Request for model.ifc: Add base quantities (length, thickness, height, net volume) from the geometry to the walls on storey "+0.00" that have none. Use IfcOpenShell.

First a look at what the model holds.

```python
import ifcopenshell
import ifcopenshell.util.element
import ifcopenshell.util.unit

model = ifcopenshell.open("model.ifc")
print(model.schema)
for unit_type in ("LENGTHUNIT", "AREAUNIT", "VOLUMEUNIT"):
    print(unit_type, ifcopenshell.util.unit.calculate_unit_scale(model, unit_type))
storey = next(s for s in model.by_type("IfcBuildingStorey") if s.Name == "+0.00")
walls = [e for e in ifcopenshell.util.element.get_decomposition(storey) if e.is_a("IfcWall")]
for e in sorted(walls, key=lambda e: e.id()):
    print(e.id(), e.is_a(), e.Name, list(ifcopenshell.util.element.get_psets(e, qtos_only=True)), sep=" | ")
```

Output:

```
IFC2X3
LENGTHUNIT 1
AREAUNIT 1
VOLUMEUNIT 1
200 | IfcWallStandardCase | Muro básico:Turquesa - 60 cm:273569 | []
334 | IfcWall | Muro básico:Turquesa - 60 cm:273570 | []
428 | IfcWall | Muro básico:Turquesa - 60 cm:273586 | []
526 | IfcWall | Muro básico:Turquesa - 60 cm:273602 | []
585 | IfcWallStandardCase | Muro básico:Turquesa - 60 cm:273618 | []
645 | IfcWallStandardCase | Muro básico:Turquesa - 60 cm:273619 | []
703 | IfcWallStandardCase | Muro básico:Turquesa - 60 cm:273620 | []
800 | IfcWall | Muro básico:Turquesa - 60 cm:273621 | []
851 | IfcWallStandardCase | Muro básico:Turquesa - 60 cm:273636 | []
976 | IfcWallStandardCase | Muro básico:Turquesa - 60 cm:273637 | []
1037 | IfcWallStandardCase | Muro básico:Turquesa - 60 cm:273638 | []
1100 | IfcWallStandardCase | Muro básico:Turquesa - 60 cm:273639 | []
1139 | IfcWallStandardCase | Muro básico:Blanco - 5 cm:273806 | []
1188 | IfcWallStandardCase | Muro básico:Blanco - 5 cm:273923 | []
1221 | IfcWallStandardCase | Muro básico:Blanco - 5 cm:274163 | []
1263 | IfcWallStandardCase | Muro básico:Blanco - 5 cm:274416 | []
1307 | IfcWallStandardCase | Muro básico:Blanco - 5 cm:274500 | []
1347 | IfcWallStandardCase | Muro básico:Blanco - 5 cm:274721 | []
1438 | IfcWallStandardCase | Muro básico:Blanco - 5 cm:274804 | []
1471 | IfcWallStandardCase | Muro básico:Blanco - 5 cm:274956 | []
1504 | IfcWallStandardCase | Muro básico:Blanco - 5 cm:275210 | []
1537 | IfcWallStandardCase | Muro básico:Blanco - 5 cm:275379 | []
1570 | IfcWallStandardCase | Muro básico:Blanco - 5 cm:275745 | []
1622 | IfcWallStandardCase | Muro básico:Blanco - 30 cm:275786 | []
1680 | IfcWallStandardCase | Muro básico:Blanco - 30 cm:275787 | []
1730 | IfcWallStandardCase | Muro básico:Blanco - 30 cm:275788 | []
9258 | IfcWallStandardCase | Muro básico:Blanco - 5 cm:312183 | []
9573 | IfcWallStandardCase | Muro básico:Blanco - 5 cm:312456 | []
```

```python
import ifcopenshell
import ifcopenshell.api.pset
import ifcopenshell.geom
import ifcopenshell.util.element
import ifcopenshell.util.shape
import ifcopenshell.util.unit

model = ifcopenshell.open("model.ifc")
unit_scale = ifcopenshell.util.unit.calculate_unit_scale(model)
volume_scale = ifcopenshell.util.unit.calculate_unit_scale(model, "VOLUMEUNIT")
settings = ifcopenshell.geom.settings()

storey = next(s for s in model.by_type("IfcBuildingStorey") if s.Name == "+0.00")
walls = [e for e in ifcopenshell.util.element.get_decomposition(storey) if e.is_a("IfcWall")]

for e in sorted(walls, key=lambda e: e.id()):
    if ifcopenshell.util.element.get_psets(e, qtos_only=True, should_inherit=False):
        continue
    # Geometry comes back in metres, in the element's own axes.
    shape = ifcopenshell.geom.create_shape(settings, e)
    values = {
        "Length": ifcopenshell.util.shape.get_x(shape.geometry) / unit_scale,
        "Width": ifcopenshell.util.shape.get_y(shape.geometry) / unit_scale,
        "Height": ifcopenshell.util.shape.get_z(shape.geometry) / unit_scale,
        "NetVolume": ifcopenshell.util.shape.get_volume(shape.geometry) / volume_scale,
    }
    qto = ifcopenshell.api.pset.add_qto(model, product=e, name="BaseQuantities")
    ifcopenshell.api.pset.edit_qto(model, qto=qto, properties=values)
    print(e.id(), {k: round(v, 3) for k, v in values.items()})

model.write("model_edited.ifc")
```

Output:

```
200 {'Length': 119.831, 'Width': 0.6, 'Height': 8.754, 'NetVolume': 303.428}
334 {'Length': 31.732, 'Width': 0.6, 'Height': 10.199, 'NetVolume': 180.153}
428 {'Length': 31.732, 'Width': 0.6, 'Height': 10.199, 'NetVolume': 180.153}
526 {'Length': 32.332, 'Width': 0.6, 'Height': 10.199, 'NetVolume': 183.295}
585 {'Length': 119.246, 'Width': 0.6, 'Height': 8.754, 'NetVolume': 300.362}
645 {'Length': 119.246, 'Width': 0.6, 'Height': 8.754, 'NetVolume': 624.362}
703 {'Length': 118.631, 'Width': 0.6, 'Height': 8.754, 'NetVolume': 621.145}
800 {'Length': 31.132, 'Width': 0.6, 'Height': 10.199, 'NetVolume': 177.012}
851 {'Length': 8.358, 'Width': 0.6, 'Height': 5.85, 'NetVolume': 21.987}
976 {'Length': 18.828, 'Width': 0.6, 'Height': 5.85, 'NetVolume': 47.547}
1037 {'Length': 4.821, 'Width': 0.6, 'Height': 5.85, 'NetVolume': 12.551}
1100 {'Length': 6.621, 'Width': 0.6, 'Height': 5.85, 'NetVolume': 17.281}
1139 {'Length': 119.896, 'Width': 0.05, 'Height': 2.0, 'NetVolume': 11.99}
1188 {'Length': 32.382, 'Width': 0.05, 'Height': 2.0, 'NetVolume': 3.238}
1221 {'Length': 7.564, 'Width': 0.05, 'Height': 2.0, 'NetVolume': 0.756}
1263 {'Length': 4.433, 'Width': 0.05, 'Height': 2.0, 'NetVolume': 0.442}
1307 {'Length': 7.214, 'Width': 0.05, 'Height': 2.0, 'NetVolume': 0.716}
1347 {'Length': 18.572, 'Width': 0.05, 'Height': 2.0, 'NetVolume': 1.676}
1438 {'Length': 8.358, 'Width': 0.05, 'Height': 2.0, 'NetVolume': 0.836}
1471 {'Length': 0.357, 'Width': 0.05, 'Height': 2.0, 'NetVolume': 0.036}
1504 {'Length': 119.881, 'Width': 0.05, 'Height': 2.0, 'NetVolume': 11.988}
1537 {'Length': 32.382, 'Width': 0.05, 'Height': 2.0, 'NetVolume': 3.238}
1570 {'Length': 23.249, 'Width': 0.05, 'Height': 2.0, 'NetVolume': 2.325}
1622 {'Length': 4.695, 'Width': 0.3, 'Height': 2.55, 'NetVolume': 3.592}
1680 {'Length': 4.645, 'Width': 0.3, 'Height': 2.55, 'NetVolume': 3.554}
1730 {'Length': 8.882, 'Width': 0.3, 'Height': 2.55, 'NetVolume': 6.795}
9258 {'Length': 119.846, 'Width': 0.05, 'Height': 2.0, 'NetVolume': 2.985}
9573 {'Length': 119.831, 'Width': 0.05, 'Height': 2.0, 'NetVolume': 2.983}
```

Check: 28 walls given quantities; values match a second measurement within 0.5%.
